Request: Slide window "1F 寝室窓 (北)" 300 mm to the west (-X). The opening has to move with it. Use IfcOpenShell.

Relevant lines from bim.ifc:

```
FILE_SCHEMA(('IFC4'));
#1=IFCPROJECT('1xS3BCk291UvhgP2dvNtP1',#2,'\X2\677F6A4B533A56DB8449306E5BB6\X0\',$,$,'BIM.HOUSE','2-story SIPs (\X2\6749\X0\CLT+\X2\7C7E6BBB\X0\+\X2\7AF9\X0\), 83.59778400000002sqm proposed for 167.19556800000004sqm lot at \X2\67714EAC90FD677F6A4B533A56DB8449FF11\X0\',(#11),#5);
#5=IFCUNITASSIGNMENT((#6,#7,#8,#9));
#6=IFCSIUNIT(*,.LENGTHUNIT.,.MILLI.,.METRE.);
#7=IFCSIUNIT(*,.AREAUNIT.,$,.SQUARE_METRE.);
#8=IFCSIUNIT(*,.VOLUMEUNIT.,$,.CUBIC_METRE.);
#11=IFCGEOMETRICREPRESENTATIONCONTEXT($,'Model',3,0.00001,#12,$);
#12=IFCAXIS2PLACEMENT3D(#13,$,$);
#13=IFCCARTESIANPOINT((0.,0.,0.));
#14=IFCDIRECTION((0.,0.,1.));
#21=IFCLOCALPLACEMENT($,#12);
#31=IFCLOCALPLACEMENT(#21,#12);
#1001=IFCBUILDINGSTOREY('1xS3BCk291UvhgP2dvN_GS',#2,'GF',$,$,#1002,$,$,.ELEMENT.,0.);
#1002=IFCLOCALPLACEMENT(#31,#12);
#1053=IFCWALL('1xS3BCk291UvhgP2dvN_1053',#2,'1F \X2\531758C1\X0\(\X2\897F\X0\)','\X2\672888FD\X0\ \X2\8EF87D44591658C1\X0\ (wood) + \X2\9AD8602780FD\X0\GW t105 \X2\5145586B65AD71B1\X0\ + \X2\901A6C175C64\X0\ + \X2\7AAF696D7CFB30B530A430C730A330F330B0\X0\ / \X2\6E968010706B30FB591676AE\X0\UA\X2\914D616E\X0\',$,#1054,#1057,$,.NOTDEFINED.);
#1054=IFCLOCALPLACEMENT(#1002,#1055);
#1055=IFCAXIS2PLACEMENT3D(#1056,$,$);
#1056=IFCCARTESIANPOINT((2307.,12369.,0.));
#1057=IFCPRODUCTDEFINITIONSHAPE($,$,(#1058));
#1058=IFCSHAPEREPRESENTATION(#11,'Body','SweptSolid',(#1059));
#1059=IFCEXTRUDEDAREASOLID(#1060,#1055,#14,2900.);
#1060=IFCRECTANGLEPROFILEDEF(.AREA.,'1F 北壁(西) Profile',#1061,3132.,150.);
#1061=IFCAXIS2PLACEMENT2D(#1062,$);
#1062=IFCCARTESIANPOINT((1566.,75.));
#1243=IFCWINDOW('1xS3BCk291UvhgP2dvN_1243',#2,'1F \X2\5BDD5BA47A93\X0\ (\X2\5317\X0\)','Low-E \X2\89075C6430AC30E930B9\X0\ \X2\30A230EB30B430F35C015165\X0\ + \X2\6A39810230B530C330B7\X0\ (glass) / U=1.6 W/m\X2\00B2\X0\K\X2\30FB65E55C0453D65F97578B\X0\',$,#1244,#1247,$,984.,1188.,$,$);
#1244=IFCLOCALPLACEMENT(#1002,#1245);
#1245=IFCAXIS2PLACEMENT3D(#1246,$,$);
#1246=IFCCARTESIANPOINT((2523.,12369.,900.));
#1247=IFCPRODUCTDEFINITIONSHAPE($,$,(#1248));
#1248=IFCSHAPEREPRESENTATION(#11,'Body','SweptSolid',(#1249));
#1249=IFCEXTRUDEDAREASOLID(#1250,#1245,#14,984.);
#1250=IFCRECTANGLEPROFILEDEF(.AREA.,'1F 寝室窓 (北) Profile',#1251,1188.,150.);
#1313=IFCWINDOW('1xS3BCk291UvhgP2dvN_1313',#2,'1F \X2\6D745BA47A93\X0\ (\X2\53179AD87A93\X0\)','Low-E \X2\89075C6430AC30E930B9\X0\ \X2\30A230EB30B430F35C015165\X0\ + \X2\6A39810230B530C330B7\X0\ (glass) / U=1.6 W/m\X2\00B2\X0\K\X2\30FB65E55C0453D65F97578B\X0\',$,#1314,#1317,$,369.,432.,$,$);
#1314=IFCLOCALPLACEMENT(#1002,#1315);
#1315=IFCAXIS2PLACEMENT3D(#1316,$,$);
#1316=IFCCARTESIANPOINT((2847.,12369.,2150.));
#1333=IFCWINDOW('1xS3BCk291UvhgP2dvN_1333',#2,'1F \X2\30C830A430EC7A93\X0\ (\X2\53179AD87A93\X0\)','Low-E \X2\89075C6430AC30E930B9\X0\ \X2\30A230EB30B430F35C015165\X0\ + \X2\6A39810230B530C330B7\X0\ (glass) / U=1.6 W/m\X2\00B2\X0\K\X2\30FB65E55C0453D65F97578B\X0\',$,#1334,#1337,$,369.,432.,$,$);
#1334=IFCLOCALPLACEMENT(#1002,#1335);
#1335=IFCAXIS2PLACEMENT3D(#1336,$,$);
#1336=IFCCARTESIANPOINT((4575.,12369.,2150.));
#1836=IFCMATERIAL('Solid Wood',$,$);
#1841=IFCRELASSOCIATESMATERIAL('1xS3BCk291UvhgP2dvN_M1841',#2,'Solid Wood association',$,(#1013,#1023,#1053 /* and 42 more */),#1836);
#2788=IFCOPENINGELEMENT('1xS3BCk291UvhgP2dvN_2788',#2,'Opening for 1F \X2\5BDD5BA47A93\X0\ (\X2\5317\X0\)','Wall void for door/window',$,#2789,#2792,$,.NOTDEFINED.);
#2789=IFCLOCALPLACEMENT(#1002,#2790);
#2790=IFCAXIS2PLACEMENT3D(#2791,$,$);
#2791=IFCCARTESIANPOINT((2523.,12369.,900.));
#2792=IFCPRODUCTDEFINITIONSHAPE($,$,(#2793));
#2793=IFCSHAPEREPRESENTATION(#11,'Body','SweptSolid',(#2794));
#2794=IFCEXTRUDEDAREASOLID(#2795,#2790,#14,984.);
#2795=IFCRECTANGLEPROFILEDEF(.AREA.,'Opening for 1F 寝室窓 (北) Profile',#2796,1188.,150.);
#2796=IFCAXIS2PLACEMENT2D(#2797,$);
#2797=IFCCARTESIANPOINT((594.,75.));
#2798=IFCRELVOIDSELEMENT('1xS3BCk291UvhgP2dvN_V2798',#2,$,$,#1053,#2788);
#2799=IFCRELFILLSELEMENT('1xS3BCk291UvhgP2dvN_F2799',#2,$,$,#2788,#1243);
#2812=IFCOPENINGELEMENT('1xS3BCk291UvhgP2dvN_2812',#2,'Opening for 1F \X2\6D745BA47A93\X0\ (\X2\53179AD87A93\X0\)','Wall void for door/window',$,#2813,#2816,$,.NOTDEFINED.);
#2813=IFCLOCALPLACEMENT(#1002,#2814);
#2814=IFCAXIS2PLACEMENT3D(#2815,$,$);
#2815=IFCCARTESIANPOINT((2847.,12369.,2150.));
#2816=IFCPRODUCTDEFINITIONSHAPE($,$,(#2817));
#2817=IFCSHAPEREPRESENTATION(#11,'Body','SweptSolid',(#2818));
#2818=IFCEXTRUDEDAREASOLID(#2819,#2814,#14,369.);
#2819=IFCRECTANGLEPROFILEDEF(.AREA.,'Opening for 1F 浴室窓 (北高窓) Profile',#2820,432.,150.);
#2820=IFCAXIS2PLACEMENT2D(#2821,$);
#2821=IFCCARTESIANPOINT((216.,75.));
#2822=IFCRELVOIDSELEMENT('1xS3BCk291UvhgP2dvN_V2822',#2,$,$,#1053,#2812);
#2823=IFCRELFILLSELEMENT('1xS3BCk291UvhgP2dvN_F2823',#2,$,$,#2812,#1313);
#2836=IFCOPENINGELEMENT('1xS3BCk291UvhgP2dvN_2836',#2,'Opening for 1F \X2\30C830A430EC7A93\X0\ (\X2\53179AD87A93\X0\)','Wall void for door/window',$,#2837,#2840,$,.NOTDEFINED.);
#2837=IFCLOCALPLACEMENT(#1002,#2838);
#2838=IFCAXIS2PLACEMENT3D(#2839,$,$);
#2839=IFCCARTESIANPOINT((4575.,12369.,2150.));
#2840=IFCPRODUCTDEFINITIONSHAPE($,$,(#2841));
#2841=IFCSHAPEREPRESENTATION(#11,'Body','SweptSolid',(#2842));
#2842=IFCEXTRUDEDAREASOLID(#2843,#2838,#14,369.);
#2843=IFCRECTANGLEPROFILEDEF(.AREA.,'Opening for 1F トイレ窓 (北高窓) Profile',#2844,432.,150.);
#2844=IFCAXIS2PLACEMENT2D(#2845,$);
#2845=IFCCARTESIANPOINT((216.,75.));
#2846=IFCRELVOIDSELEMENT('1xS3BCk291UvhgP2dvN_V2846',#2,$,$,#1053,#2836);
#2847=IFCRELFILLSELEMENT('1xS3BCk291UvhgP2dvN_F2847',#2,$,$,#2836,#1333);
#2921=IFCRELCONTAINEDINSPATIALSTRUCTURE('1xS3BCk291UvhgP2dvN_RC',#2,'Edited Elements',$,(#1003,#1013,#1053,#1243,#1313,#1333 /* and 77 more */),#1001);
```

```python
import ifcopenshell
import ifcopenshell.api.geometry
import ifcopenshell.util.placement
import ifcopenshell.util.unit

model = ifcopenshell.open("bim.ifc")
unit_scale = ifcopenshell.util.unit.calculate_unit_scale(model)

window = model.by_guid("1xS3BCk291UvhgP2dvN_1243")
opening = window.FillsVoids[0].RelatingOpeningElement
wall = opening.VoidsElements[0].RelatingBuildingElement

wall_matrix = ifcopenshell.util.placement.get_local_placement(wall.ObjectPlacement)
shift = wall_matrix[:3, 0] * -0.3 / unit_scale
before = ifcopenshell.util.placement.get_local_placement(window.ObjectPlacement)[:3, 3].copy()

# The window is not placed relative to its opening, so move both.
for product in (opening, window):
    matrix = ifcopenshell.util.placement.get_local_placement(product.ObjectPlacement)
    matrix[:3, 3] += shift
    ifcopenshell.api.geometry.edit_object_placement(model, product=product, matrix=matrix, is_si=False)

after = ifcopenshell.util.placement.get_local_placement(window.ObjectPlacement)[:3, 3]
print("window moved by", (after - before).round(3) + 0.0)

model.write("bim-out.ifc")
```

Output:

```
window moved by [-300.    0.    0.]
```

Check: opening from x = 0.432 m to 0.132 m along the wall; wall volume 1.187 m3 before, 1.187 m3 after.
